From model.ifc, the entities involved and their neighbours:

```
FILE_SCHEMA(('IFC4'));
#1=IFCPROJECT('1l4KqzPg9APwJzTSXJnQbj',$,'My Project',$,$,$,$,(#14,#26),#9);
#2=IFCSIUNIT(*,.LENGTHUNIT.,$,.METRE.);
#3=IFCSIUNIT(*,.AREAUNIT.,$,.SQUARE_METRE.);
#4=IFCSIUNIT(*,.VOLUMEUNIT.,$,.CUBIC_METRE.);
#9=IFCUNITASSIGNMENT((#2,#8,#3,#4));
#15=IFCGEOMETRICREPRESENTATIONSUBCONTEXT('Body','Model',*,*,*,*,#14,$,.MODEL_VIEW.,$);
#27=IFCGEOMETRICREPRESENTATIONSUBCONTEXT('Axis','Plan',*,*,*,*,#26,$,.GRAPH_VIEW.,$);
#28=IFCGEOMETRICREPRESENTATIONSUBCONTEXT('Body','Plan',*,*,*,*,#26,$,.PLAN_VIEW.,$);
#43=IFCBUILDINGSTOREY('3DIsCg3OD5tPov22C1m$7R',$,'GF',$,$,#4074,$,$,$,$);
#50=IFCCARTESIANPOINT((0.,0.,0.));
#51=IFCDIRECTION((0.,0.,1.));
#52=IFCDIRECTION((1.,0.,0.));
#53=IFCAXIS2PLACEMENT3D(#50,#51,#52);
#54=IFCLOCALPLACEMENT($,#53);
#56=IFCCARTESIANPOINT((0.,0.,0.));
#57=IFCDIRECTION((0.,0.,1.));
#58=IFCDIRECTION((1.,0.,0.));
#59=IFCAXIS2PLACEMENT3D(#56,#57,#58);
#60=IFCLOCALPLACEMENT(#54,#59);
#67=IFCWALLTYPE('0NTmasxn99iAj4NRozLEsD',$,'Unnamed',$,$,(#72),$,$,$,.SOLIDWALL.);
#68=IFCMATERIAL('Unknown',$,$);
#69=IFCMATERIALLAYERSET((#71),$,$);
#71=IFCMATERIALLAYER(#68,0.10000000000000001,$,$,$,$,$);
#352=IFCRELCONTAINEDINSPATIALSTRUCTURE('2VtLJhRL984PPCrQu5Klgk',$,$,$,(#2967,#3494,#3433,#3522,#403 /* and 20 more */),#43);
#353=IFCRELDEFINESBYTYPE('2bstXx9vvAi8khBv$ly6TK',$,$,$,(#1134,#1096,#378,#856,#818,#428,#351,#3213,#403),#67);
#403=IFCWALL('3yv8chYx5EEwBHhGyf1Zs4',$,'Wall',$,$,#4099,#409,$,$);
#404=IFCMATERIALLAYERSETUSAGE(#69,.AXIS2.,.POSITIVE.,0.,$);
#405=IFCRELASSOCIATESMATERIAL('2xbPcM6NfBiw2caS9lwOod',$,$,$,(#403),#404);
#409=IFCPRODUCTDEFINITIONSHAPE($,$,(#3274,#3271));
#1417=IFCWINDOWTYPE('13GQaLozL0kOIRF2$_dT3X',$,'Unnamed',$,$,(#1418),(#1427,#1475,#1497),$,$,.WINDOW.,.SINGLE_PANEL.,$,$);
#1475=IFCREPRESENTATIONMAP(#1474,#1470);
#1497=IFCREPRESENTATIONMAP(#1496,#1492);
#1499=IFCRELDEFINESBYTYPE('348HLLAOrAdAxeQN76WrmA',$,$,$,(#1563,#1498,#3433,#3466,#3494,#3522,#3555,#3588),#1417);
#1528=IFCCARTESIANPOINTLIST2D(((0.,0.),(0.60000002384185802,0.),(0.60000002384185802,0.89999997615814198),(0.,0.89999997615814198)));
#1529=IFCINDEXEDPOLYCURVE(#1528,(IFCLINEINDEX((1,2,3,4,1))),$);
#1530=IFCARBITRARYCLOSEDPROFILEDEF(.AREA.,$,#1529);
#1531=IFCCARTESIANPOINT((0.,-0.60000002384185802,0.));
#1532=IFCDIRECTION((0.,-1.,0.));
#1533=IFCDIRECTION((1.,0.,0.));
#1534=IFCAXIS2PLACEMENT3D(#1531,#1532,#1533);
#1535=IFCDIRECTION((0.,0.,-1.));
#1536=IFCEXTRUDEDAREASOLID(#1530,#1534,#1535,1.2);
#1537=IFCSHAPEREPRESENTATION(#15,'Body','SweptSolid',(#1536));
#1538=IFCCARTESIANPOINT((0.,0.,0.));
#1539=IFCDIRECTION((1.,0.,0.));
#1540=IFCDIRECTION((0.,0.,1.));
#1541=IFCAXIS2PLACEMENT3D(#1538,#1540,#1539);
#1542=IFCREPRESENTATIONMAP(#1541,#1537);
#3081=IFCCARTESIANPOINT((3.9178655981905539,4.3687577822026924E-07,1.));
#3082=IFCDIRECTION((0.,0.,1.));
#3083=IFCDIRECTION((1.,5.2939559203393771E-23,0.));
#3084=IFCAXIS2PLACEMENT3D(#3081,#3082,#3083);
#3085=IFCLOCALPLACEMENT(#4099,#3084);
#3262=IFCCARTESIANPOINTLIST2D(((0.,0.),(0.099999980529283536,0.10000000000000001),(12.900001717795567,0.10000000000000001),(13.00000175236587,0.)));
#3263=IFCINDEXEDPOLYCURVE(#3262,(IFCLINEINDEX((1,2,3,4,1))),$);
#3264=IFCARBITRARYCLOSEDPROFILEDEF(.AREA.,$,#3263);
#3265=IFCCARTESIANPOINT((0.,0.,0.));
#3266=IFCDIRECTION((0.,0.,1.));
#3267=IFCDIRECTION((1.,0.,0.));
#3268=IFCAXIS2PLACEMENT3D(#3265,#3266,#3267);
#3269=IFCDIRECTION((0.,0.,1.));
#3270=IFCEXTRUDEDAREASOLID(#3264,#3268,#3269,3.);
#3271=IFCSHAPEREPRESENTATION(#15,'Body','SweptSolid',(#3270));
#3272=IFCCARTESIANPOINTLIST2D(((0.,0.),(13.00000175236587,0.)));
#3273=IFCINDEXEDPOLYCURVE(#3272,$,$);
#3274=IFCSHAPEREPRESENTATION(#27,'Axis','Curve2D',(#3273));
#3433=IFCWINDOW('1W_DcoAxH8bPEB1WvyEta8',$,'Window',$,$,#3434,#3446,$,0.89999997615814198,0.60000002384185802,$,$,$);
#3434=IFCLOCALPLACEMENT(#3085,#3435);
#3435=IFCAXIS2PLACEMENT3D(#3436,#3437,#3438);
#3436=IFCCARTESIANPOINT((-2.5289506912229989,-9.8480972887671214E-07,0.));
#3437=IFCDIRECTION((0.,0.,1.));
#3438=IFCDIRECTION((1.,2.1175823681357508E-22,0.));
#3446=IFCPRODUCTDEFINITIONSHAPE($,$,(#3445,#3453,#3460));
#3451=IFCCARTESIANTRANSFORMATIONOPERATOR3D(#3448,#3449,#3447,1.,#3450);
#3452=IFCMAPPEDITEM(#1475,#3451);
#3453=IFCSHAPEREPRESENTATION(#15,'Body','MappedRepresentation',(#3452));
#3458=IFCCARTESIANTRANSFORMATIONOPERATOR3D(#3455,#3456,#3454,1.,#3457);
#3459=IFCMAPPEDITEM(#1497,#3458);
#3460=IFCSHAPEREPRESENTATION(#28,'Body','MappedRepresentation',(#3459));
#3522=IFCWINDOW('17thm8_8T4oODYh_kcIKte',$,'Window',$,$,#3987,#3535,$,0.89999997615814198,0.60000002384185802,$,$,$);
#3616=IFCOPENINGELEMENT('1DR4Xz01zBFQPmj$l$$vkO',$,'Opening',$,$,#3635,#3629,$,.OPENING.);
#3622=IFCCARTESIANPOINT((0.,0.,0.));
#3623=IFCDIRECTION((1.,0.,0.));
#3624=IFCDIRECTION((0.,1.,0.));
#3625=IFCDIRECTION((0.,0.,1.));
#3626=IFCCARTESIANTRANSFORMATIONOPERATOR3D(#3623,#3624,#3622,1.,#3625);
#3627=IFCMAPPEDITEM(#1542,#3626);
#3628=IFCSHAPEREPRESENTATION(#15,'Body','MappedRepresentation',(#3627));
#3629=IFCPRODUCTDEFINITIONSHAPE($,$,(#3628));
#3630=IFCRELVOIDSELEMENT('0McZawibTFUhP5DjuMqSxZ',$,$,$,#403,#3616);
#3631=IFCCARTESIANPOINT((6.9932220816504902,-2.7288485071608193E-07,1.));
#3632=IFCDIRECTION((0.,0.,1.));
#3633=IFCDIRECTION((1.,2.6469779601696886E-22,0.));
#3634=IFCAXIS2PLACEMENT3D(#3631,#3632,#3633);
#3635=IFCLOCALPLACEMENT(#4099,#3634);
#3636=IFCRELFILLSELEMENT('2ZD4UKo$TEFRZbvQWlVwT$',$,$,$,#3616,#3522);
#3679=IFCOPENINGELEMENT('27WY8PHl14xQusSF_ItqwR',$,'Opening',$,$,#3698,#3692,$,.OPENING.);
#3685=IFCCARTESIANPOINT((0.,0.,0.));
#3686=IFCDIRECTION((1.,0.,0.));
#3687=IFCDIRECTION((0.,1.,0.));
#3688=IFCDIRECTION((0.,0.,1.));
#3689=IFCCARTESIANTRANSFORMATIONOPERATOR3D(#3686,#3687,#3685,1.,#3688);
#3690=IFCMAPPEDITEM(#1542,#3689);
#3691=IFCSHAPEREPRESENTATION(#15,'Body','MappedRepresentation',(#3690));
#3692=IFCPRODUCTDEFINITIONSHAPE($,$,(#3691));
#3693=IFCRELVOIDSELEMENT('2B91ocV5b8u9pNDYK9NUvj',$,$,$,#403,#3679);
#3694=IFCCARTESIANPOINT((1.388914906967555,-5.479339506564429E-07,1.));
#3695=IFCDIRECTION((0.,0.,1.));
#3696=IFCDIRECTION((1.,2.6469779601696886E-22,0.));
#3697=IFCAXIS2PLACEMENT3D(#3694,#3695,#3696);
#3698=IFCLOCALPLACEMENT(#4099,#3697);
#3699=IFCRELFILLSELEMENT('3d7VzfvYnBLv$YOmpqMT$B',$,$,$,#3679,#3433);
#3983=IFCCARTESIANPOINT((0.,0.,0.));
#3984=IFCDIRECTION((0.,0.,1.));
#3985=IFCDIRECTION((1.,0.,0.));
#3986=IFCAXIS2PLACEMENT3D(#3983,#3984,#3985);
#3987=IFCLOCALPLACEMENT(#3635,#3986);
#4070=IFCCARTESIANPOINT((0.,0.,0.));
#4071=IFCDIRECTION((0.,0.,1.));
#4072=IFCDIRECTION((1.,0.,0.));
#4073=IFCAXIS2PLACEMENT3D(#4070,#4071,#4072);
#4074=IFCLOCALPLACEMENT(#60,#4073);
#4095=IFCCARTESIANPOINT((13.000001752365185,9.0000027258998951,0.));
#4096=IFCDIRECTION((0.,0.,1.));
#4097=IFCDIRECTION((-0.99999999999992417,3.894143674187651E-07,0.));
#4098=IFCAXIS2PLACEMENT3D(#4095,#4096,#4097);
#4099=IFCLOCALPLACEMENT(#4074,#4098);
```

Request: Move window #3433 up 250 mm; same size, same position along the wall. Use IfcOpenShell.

```python
import numpy as np
import ifcopenshell
import ifcopenshell.api.geometry
import ifcopenshell.util.placement
import ifcopenshell.util.unit

model = ifcopenshell.open("model.ifc")
unit_scale = ifcopenshell.util.unit.calculate_unit_scale(model)

window = model.by_id(3433)
opening = window.FillsVoids[0].RelatingOpeningElement
dz = 0.25 / unit_scale

shift = np.array([0.0, 0.0, dz])
# The window is not placed relative to its opening, so move both.
for product in (opening, window):
    matrix = ifcopenshell.util.placement.get_local_placement(product.ObjectPlacement)
    matrix[:3, 3] += shift
    ifcopenshell.api.geometry.edit_object_placement(model, product=product, matrix=matrix, is_si=False)

print(f"moved by {dz * unit_scale:+.3f} m")

model.write("model_rev.ifc")
```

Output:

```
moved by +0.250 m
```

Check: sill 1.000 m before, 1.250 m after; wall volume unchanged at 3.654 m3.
